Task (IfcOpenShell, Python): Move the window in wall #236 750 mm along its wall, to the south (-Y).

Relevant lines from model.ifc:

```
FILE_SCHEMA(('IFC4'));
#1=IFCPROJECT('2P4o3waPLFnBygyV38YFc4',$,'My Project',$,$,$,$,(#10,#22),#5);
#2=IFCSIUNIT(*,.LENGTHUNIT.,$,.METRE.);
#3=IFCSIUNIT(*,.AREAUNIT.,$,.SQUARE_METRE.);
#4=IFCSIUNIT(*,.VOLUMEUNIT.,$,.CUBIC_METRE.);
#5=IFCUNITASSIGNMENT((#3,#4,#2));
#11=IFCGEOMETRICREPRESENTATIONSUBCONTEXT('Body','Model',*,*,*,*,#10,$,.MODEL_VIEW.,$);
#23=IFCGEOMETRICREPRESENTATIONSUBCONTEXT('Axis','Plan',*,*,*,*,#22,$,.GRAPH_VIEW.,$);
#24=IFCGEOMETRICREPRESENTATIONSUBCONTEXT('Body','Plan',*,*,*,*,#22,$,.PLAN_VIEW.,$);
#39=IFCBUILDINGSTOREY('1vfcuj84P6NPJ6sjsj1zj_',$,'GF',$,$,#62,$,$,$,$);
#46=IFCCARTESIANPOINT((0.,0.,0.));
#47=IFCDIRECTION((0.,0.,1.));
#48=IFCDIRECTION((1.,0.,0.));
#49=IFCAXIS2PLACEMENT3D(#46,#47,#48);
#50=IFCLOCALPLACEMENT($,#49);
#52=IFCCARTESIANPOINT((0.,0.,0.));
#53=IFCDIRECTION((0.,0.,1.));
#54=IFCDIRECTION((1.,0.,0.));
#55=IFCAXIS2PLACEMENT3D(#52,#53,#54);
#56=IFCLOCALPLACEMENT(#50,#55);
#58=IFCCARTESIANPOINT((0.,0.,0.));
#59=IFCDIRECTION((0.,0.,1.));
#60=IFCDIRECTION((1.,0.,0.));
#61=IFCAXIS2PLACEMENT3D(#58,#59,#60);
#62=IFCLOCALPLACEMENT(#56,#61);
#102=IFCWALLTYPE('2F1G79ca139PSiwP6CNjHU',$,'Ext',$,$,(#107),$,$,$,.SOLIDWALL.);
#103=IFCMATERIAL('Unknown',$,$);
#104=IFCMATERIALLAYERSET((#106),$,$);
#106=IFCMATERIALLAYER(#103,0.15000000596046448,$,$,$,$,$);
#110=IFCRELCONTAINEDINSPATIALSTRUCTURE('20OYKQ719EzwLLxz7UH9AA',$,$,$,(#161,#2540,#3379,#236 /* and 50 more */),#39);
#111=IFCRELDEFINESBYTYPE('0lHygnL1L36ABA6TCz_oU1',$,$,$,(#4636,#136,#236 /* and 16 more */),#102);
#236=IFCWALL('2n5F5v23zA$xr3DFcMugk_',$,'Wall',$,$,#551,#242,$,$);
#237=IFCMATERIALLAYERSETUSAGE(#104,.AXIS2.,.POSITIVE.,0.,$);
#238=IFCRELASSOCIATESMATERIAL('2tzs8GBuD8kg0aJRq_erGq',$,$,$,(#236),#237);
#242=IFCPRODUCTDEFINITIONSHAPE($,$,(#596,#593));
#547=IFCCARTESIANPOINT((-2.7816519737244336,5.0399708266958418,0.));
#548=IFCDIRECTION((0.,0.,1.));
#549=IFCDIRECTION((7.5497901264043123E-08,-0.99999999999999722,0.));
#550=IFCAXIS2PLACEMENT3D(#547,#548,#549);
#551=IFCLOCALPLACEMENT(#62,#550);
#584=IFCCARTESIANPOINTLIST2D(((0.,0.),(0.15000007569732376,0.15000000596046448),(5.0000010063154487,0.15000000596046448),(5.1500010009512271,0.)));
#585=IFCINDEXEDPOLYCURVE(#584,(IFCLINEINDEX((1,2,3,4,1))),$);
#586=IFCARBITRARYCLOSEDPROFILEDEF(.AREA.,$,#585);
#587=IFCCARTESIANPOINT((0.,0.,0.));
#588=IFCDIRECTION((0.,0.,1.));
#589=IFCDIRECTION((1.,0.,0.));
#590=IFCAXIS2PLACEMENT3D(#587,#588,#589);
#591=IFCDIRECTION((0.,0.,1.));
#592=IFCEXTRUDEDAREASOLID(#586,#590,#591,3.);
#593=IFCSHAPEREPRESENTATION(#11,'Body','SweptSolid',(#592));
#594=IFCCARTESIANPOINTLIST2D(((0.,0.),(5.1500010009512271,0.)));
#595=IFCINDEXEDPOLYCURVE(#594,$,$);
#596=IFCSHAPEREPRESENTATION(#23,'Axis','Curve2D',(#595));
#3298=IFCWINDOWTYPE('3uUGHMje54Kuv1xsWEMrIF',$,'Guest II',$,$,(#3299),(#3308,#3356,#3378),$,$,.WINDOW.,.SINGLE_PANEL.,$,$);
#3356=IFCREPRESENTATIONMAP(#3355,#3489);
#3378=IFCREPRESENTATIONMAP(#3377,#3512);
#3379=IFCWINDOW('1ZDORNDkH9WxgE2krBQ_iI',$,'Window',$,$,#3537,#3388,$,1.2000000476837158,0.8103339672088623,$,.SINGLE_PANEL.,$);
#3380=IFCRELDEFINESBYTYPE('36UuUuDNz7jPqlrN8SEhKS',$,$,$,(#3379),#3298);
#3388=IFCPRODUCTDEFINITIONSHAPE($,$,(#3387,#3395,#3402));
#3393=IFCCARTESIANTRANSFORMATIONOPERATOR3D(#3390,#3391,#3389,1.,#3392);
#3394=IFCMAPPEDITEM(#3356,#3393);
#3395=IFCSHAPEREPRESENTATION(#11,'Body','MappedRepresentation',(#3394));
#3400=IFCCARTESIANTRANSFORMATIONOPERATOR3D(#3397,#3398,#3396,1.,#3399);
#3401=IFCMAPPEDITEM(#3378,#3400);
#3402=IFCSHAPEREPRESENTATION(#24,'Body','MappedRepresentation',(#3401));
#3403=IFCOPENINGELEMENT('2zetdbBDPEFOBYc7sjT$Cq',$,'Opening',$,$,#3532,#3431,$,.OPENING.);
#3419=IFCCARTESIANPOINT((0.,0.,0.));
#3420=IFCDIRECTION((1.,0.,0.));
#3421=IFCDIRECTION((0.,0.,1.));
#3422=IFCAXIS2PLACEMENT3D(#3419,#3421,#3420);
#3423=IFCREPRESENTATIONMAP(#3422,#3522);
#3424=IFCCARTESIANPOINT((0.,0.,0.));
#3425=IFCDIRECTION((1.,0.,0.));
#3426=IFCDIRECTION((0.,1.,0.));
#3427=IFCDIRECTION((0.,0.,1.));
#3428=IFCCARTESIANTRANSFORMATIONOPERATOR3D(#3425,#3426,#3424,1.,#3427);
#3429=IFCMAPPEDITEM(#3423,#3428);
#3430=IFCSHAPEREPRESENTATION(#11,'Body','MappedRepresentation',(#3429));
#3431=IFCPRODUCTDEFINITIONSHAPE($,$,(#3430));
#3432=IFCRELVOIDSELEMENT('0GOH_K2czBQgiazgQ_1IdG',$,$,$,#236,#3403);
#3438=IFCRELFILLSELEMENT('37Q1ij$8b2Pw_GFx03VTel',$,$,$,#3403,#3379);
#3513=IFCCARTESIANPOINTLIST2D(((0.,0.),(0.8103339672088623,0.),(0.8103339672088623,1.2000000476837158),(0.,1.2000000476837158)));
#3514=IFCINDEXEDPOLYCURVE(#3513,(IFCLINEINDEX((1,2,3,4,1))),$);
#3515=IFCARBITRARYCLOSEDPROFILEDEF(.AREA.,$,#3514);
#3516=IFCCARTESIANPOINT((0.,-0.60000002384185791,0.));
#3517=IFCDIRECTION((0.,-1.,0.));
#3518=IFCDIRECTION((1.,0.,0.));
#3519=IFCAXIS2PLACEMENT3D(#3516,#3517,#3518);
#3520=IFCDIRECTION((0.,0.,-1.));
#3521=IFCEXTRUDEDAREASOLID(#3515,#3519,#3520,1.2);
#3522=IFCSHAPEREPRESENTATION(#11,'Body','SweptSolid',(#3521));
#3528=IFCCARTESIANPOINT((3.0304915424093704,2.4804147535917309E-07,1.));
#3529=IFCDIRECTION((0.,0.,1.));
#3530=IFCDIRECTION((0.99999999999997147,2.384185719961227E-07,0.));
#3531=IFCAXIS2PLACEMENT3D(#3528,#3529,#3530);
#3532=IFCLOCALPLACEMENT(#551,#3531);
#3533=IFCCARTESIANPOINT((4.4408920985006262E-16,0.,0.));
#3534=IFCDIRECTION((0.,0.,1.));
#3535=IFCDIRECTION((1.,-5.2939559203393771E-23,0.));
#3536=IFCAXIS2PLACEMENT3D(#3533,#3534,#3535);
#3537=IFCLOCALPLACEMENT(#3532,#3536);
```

```python
import ifcopenshell
import ifcopenshell.api.geometry
import ifcopenshell.util.placement
import ifcopenshell.util.unit

model = ifcopenshell.open("model.ifc")
unit_scale = ifcopenshell.util.unit.calculate_unit_scale(model)

window = model.by_guid("1ZDORNDkH9WxgE2krBQ_iI")
opening = window.FillsVoids[0].RelatingOpeningElement
wall = opening.VoidsElements[0].RelatingBuildingElement

wall_matrix = ifcopenshell.util.placement.get_local_placement(wall.ObjectPlacement)
shift = wall_matrix[:3, 0] * 0.75 / unit_scale
before = ifcopenshell.util.placement.get_local_placement(window.ObjectPlacement)[:3, 3].copy()

# The window is placed relative to its opening, so it follows when the opening moves.
matrix = ifcopenshell.util.placement.get_local_placement(opening.ObjectPlacement)
matrix[:3, 3] += shift
ifcopenshell.api.geometry.edit_object_placement(
    model, product=opening, matrix=matrix, is_si=False, should_transform_children=True
)

after = ifcopenshell.util.placement.get_local_placement(window.ObjectPlacement)[:3, 3]
print("window moved by", (after - before).round(3) + 0.0)

model.write("model_updated.ifc")
```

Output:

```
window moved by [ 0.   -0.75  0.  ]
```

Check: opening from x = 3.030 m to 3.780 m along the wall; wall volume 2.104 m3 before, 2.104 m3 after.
